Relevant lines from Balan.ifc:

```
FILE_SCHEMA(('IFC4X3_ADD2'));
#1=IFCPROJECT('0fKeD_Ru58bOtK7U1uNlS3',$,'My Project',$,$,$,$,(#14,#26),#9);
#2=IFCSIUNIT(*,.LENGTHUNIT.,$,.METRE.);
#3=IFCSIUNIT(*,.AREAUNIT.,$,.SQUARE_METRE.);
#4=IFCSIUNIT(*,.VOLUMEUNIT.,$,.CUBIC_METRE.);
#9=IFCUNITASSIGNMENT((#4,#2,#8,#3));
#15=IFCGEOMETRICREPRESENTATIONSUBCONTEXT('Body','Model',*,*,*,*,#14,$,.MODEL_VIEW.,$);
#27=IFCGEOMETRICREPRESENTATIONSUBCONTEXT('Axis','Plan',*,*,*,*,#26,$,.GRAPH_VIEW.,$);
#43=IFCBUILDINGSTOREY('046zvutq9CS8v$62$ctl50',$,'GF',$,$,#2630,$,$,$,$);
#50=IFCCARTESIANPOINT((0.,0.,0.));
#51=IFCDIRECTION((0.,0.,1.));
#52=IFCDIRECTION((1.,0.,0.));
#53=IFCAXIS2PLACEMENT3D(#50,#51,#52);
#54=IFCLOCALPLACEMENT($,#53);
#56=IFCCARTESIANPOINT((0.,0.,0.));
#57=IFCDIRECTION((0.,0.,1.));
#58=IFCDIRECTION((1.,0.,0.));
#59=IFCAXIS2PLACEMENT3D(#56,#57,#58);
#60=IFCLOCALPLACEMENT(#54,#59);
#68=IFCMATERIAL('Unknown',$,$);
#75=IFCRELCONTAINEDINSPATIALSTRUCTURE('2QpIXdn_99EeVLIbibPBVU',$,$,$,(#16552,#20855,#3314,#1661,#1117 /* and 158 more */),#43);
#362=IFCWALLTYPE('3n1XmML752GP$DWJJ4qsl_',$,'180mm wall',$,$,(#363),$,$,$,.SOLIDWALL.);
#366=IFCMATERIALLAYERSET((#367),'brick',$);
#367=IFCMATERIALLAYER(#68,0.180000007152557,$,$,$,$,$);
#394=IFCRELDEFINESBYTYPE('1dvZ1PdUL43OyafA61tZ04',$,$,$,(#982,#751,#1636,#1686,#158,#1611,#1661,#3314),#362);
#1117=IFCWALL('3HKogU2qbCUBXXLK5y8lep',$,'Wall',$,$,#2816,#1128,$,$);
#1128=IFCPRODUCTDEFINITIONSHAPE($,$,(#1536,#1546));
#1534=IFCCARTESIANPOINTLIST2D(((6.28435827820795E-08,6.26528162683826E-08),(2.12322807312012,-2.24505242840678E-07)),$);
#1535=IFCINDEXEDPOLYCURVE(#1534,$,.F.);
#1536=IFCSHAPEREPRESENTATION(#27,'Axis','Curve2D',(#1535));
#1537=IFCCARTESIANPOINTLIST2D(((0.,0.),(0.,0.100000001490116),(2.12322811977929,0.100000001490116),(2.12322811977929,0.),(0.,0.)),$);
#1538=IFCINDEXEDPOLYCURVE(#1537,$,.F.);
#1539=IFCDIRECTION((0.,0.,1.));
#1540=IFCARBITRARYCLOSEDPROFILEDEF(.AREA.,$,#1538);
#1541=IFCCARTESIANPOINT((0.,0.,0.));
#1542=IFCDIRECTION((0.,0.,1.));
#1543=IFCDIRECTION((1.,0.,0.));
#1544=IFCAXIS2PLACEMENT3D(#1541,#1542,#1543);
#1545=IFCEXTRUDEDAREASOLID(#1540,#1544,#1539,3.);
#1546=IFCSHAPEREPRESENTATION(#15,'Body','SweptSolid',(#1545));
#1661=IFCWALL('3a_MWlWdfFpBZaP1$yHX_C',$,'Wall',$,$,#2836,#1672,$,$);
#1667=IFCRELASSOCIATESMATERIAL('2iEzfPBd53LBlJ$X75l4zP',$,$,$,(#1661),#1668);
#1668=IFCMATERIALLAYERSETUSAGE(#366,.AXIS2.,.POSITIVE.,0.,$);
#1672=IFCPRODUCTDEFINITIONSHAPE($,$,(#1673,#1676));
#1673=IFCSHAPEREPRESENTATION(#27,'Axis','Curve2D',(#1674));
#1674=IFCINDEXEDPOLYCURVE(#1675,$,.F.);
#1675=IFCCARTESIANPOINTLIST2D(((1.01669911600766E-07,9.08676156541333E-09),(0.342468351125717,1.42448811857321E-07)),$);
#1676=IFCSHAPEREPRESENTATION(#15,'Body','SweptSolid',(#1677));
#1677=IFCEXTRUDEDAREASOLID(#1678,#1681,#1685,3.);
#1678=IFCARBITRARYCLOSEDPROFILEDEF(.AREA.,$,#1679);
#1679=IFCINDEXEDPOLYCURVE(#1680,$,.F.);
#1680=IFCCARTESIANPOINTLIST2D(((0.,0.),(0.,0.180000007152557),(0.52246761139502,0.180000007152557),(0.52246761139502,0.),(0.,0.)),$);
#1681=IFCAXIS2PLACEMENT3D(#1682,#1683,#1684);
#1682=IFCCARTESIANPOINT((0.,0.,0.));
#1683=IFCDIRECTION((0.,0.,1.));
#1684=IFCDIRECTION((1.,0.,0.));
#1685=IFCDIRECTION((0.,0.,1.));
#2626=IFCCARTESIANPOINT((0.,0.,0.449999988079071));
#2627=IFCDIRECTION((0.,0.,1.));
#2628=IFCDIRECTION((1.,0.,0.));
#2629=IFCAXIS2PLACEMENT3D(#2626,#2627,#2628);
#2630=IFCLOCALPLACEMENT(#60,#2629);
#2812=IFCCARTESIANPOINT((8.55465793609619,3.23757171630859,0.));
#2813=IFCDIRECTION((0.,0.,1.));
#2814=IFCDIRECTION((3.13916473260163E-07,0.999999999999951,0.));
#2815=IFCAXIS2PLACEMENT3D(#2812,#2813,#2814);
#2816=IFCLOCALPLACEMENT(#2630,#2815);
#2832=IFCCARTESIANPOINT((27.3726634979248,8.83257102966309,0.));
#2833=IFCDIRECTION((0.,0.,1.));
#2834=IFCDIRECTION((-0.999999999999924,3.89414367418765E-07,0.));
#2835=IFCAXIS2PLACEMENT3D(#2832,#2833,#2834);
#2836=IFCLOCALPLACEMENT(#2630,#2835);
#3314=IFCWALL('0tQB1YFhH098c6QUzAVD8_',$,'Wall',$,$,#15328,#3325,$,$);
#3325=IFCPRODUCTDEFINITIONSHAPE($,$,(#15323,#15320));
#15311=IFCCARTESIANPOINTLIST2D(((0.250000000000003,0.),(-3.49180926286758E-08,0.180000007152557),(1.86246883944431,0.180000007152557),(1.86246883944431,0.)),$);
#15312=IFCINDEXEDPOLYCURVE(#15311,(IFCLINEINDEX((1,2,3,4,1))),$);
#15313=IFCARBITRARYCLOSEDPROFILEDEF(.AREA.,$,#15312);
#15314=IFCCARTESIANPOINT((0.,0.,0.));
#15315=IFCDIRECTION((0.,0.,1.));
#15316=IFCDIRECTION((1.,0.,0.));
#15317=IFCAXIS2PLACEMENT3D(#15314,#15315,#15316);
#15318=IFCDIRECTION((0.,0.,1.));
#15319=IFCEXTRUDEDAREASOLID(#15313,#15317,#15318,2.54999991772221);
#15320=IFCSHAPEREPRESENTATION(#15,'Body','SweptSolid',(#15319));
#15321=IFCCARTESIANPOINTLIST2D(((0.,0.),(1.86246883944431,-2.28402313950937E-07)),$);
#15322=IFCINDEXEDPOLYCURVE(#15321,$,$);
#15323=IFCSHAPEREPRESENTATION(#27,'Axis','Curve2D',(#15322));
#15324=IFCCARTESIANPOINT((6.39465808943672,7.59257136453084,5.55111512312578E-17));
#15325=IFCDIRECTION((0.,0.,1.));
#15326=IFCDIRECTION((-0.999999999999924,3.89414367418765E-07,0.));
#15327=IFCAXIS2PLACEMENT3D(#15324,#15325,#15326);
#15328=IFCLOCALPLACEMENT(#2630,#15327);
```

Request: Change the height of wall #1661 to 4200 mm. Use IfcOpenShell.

```python
import ifcopenshell
import ifcopenshell.geom
import ifcopenshell.util.representation
import ifcopenshell.util.shape
import ifcopenshell.util.unit

model = ifcopenshell.open("Balan.ifc")
unit_scale = ifcopenshell.util.unit.calculate_unit_scale(model)
settings = ifcopenshell.geom.settings()


def volume(element):
    """Net volume in cubic metres, openings subtracted."""
    shape = ifcopenshell.geom.create_shape(settings, element)
    return ifcopenshell.util.shape.get_volume(shape.geometry)


wall = model.by_guid("3a_MWlWdfFpBZaP1$yHX_C")
before = volume(wall)

body = ifcopenshell.util.representation.get_representation(wall, "Model", "Body")
solid = body.Items[0]
old_height = solid.Depth
solid.Depth = 4.2 / unit_scale
after = volume(wall)

print(f"height {old_height:g} -> {solid.Depth:g}, volume {before:.3f} -> {after:.3f} m3")

model.write("Balan_updated.ifc")
```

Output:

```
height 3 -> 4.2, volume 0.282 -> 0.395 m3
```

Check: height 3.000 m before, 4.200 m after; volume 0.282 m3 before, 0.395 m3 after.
